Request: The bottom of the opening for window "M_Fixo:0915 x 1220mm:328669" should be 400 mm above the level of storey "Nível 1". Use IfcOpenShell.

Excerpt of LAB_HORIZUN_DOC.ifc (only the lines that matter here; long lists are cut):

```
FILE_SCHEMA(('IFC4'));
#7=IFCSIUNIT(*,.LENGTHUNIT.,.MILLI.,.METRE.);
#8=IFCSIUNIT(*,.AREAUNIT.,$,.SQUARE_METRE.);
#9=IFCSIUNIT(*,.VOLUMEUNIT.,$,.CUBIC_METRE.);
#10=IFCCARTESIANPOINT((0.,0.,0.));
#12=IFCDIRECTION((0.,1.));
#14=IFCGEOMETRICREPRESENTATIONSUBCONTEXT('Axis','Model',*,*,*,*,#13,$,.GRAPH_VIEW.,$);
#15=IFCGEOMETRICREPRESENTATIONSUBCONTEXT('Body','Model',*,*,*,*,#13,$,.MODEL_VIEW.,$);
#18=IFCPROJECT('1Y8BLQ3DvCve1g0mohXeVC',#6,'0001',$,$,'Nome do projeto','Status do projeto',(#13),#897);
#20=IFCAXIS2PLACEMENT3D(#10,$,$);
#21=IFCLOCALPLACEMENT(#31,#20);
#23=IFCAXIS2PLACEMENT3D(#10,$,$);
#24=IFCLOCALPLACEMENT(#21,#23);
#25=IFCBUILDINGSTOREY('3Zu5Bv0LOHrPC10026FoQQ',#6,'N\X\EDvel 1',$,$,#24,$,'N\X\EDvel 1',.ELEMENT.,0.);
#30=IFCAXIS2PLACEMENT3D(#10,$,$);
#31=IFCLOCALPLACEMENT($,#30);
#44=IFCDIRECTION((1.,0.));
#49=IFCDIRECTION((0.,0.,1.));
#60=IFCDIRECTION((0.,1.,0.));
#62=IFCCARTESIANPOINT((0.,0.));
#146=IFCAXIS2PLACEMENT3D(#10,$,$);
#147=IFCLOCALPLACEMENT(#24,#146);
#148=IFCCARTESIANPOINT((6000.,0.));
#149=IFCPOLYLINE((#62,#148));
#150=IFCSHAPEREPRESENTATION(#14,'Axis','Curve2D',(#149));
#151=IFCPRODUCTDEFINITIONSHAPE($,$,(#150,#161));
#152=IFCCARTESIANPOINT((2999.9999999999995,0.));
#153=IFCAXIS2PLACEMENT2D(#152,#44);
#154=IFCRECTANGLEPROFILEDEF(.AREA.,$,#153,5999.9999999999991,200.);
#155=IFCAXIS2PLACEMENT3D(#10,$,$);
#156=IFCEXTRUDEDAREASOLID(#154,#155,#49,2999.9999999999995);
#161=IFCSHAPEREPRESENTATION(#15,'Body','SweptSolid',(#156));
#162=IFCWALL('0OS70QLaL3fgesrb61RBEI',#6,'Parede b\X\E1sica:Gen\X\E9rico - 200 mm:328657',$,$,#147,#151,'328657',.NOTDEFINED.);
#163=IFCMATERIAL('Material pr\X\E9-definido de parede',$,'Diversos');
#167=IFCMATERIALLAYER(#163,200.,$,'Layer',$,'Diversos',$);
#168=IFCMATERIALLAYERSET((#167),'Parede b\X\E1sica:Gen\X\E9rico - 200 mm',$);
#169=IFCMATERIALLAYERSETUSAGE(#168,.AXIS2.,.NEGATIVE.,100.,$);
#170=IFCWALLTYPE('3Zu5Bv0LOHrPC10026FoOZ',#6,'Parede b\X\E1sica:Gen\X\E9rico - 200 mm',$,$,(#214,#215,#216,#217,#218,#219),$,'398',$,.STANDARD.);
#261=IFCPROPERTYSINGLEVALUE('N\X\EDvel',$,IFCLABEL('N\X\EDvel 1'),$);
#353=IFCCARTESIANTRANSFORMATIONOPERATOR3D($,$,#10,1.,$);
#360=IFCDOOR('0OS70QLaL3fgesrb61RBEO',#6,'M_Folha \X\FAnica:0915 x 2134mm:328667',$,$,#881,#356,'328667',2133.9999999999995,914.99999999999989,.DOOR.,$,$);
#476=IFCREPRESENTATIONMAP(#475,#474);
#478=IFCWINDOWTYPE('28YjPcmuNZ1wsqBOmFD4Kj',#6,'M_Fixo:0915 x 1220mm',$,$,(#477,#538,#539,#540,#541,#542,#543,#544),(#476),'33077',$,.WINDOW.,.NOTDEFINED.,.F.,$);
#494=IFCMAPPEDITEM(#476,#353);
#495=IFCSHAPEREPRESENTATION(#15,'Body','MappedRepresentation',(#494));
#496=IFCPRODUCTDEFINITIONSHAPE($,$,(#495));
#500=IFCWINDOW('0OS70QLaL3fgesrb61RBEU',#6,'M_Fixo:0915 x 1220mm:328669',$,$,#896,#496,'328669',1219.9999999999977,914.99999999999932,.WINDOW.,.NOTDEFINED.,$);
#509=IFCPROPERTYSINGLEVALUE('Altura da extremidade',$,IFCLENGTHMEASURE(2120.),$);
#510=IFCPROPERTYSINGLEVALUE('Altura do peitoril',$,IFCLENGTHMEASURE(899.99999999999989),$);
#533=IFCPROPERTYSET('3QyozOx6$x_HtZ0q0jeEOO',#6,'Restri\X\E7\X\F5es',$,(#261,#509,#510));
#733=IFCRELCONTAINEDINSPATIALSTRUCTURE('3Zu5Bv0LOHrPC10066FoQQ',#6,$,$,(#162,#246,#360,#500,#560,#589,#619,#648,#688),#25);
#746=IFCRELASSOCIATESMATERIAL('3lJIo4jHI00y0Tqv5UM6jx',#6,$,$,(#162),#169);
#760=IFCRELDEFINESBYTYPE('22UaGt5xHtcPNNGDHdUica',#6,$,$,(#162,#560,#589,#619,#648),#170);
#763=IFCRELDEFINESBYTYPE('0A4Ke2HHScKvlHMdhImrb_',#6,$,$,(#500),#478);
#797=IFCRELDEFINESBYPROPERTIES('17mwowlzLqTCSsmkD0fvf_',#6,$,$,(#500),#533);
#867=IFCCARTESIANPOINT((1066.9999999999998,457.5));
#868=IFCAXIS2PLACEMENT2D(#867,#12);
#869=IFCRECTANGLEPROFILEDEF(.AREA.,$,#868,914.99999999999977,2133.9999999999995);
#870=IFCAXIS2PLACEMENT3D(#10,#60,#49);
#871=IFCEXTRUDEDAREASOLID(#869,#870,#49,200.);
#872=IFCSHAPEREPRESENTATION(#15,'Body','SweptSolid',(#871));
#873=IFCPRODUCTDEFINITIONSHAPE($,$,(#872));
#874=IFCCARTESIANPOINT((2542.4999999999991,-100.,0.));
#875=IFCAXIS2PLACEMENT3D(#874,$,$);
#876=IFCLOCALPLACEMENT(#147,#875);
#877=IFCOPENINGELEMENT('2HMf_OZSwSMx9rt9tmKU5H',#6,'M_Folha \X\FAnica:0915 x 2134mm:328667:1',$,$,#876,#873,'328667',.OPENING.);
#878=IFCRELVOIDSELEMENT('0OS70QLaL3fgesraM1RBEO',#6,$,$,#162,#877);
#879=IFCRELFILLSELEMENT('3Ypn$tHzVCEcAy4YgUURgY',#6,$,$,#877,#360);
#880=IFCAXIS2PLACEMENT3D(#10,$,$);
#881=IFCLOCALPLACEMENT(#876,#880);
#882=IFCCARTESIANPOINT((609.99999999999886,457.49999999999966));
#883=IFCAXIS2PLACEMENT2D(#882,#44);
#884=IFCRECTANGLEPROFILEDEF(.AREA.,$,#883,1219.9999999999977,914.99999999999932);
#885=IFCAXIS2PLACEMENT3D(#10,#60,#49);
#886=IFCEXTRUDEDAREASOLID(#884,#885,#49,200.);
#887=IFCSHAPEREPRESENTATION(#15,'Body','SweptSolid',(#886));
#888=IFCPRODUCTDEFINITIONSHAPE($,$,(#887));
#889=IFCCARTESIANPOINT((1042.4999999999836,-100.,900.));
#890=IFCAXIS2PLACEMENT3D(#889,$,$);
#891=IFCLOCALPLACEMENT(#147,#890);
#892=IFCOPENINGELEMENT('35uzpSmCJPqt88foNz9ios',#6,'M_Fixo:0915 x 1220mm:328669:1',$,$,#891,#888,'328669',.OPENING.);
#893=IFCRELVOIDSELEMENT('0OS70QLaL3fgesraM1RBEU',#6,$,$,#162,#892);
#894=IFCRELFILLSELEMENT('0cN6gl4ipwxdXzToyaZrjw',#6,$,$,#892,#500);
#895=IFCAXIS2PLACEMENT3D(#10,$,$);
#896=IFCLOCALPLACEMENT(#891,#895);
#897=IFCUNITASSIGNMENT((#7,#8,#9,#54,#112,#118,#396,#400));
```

```python
import numpy as np
import ifcopenshell
import ifcopenshell.api.geometry
import ifcopenshell.api.pset
import ifcopenshell.geom
import ifcopenshell.util.element
import ifcopenshell.util.placement
import ifcopenshell.util.shape
import ifcopenshell.util.unit

model = ifcopenshell.open("LAB_HORIZUN_DOC.ifc")
unit_scale = ifcopenshell.util.unit.calculate_unit_scale(model)

window = model.by_guid("0OS70QLaL3fgesrb61RBEU")
opening = window.FillsVoids[0].RelatingOpeningElement
storey = ifcopenshell.util.element.get_container(window, ifc_class="IfcBuildingStorey")
level = ifcopenshell.util.placement.get_local_placement(storey.ObjectPlacement)[2, 3]

# The opening's origin need not be at the sill, so measure its lowest point.
shape = ifcopenshell.geom.create_shape(ifcopenshell.geom.settings(), opening)
bottom = ifcopenshell.util.shape.get_shape_bottom_elevation(shape, shape.geometry) / unit_scale
dz = level + 0.4 / unit_scale - bottom

shift = np.array([0.0, 0.0, dz])
# The window is placed relative to its opening, so it follows when the opening moves.
matrix = ifcopenshell.util.placement.get_local_placement(opening.ObjectPlacement)
matrix[:3, 3] += shift
ifcopenshell.api.geometry.edit_object_placement(
    model, product=opening, matrix=matrix, is_si=False, should_transform_children=True
)

# Keep the stored heights in step.
pset = model.by_id(ifcopenshell.util.element.get_pset(window, "Restrições", should_inherit=False)["id"])
ifcopenshell.api.pset.edit_pset(model, pset=pset, properties={
    "Altura da extremidade": model.create_entity("IfcLengthMeasure", ifcopenshell.util.element.get_pset(window, "Restrições", "Altura da extremidade") + dz),
    "Altura do peitoril": model.create_entity("IfcLengthMeasure", ifcopenshell.util.element.get_pset(window, "Restrições", "Altura do peitoril") + dz),
})

print(f"moved by {dz * unit_scale:+.3f} m")

model.write("LAB_HORIZUN_DOC_updated.ifc")
```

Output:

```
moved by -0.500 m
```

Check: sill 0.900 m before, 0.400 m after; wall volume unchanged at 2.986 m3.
